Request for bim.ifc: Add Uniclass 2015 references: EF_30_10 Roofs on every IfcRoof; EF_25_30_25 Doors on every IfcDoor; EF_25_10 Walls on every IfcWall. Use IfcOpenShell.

First a look at what the model holds.

```python
import ifcopenshell

model = ifcopenshell.open("bim.ifc")
print(model.schema)
print("classifications:", [c.Name for c in model.by_type("IfcClassification")])
for ifc_class in ("IfcDoor", "IfcRoof", "IfcStair", "IfcWall", "IfcWindow"):
    print(ifc_class, len(model.by_type(ifc_class)))
```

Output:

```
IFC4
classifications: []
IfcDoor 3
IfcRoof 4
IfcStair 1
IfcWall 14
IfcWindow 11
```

```python
import ifcopenshell
import ifcopenshell.api.classification

model = ifcopenshell.open("bim.ifc")

system = ifcopenshell.api.classification.add_classification(model, classification="Uniclass 2015")

codes = {
    "IfcRoof": ("EF_30_10", "Roofs"),
    "IfcDoor": ("EF_25_30_25", "Doors"),
    "IfcWall": ("EF_25_10", "Walls"),
}
for ifc_class, (code, name) in codes.items():
    products = model.by_type(ifc_class)
    ifcopenshell.api.classification.add_reference(
        model, products=products, classification=system, identification=code, name=name
    )
    print(code, len(products))

model.write("bim_v2.ifc")
```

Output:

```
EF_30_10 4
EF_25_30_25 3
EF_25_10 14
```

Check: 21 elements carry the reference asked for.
